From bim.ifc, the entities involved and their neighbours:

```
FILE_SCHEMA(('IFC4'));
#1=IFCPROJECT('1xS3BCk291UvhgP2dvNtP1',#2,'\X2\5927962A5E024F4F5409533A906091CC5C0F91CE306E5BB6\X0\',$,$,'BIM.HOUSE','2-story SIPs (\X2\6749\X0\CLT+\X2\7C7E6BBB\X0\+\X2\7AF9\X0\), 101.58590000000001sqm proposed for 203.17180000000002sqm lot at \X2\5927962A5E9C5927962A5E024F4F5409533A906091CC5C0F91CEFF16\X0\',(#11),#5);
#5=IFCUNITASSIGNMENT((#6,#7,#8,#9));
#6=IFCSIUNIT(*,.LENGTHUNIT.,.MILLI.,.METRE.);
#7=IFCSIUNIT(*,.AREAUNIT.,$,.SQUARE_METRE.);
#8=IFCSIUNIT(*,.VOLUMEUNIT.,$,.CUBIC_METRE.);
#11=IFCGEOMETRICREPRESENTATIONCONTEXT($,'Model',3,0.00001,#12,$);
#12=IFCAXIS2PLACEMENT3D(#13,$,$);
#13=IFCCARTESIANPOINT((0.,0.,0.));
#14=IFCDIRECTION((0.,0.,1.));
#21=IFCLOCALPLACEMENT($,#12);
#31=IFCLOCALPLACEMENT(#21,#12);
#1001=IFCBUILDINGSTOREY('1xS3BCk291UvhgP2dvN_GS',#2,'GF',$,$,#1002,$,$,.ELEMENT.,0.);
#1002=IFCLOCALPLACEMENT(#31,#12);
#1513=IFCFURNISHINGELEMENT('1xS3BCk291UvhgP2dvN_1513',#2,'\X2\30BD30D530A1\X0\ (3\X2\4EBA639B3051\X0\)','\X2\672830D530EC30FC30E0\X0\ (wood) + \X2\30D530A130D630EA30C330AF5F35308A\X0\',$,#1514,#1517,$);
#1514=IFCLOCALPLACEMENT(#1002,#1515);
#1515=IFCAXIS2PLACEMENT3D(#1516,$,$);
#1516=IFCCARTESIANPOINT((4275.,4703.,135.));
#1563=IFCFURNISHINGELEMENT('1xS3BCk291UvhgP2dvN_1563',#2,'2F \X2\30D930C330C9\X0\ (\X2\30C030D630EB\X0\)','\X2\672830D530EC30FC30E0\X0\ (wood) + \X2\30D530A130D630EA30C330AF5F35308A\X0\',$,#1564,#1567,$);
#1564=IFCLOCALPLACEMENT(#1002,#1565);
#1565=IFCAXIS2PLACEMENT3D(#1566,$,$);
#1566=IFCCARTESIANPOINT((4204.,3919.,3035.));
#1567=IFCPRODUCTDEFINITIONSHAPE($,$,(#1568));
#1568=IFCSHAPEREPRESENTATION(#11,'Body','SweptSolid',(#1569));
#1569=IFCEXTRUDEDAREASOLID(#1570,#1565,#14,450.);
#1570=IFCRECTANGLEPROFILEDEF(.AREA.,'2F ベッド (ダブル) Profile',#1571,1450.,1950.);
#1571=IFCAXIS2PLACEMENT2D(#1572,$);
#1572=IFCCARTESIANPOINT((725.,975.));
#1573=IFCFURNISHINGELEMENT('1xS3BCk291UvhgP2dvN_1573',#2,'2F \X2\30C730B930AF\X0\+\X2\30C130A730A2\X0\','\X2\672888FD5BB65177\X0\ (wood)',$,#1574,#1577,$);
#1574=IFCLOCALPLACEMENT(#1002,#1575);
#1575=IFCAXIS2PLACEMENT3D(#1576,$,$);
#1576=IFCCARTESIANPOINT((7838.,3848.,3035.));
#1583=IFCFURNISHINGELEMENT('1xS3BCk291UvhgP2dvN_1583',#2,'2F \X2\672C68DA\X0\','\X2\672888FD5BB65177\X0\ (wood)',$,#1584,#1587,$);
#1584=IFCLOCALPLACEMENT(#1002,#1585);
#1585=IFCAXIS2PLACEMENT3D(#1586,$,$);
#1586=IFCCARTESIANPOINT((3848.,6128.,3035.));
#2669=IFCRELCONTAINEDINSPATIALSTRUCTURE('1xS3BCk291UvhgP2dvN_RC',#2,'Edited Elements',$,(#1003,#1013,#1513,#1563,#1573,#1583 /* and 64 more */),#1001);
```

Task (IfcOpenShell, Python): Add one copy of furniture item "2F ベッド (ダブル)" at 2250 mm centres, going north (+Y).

```python
import numpy as np
import ifcopenshell
import ifcopenshell.api.geometry
import ifcopenshell.api.root
import ifcopenshell.util.element
import ifcopenshell.util.placement
import ifcopenshell.util.unit

model = ifcopenshell.open("bim.ifc")
unit_scale = ifcopenshell.util.unit.calculate_unit_scale(model)


def reuse_history(source, copy):
    """copy_class also copies each property set's owner history, people and application; keep the originals."""
    for rel in copy.IsDefinedBy:
        if rel.is_a("IfcRelDefinesByProperties") and (history := rel.RelatingPropertyDefinition.OwnerHistory):
            rel.RelatingPropertyDefinition.OwnerHistory = source.OwnerHistory
            ifcopenshell.util.element.remove_deep2(model, history)


source = model.by_id(1563)
base = ifcopenshell.util.placement.get_local_placement(source.ObjectPlacement)
step = np.array([0.0, 1.0, 0.0]) * 2.25 / unit_scale

for i in range(1, 2):
    copy = ifcopenshell.api.root.copy_class(model, product=source)
    copy.Representation = ifcopenshell.util.element.copy_deep(
        model, source.Representation, exclude=["IfcGeometricRepresentationContext", "IfcRepresentationMap"]
    )
    reuse_history(source, copy)
    matrix = base.copy()
    matrix[:3, 3] += i * step
    print("added at", matrix[:3, 3].round(3) + 0.0)
    ifcopenshell.api.geometry.edit_object_placement(model, product=copy, matrix=matrix, is_si=False)

model.write("bim-out.ifc")
```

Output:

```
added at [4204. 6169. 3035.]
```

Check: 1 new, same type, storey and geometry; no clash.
